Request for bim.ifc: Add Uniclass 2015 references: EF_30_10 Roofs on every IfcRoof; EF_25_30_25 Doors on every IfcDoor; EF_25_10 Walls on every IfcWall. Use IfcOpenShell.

First a look at what the model holds.

```python
import ifcopenshell

model = ifcopenshell.open("bim.ifc")
print(model.schema)
print("classifications:", [c.Name for c in model.by_type("IfcClassification")])
for ifc_class in ("IfcDoor", "IfcRoof", "IfcStair", "IfcWall", "IfcWindow"):
    print(ifc_class, len(model.by_type(ifc_class)))
```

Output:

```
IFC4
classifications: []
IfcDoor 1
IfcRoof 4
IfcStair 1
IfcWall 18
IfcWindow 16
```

```python
import ifcopenshell
import ifcopenshell.api.classification

model = ifcopenshell.open("bim.ifc")

system = ifcopenshell.api.classification.add_classification(model, classification="Uniclass 2015")

codes = {
    "IfcRoof": ("EF_30_10", "Roofs"),
    "IfcDoor": ("EF_25_30_25", "Doors"),
    "IfcWall": ("EF_25_10", "Walls"),
}
for ifc_class, (code, name) in codes.items():
    products = model.by_type(ifc_class)
    ifcopenshell.api.classification.add_reference(
        model, products=products, classification=system, identification=code, name=name
    )
    print(code, len(products))

model.write("bim_v2.ifc")
```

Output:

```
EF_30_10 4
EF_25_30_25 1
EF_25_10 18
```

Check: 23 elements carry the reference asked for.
